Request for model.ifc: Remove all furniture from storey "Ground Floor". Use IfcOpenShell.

First a look at what the model holds.

```python
import ifcopenshell
import ifcopenshell.util.element

model = ifcopenshell.open("model.ifc")
print(model.schema)
storey = next(s for s in model.by_type("IfcBuildingStorey") if s.Name == "Ground Floor")
furniture = [e for e in ifcopenshell.util.element.get_decomposition(storey) if e.is_a("IfcFurnishingElement")]
seen = {}
for e in furniture:
    element_type = ifcopenshell.util.element.get_type(e)
    name = element_type.Name if element_type not in (None, e) else None
    seen[name] = seen.get(name, 0) + 1
for name, count in sorted(seen.items(), key=str):
    print(count, "x", name)
```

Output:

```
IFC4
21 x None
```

```python
import ifcopenshell
import ifcopenshell.api.root
import ifcopenshell.util.element

model = ifcopenshell.open("model.ifc")

storey = next(s for s in model.by_type("IfcBuildingStorey") if s.Name == "Ground Floor")
furniture = [e for e in ifcopenshell.util.element.get_decomposition(storey) if e.is_a("IfcFurnishingElement")]

for e in furniture:
    ifcopenshell.api.root.remove_product(model, product=e)
print(len(furniture), "removed")

model.write("model_edited.ifc")
```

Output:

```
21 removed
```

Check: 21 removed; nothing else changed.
